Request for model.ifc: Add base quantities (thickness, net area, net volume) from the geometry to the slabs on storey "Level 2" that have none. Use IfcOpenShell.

First a look at what the model holds.

```python
import ifcopenshell
import ifcopenshell.util.element
import ifcopenshell.util.unit

model = ifcopenshell.open("model.ifc")
print(model.schema)
for unit_type in ("LENGTHUNIT", "AREAUNIT", "VOLUMEUNIT"):
    print(unit_type, ifcopenshell.util.unit.calculate_unit_scale(model, unit_type))
storey = next(s for s in model.by_type("IfcBuildingStorey") if s.Name == "Level 2")
slabs = [e for e in ifcopenshell.util.element.get_decomposition(storey) if e.is_a("IfcSlab")]
for e in sorted(slabs, key=lambda e: e.id()):
    print(e.id(), e.is_a(), e.Name, list(ifcopenshell.util.element.get_psets(e, qtos_only=True)), sep=" | ")
```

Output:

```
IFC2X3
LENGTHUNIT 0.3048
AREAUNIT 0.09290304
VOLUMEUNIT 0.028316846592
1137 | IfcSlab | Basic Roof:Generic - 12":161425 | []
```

```python
import ifcopenshell
import ifcopenshell.api.pset
import ifcopenshell.geom
import ifcopenshell.util.element
import ifcopenshell.util.shape
import ifcopenshell.util.unit

model = ifcopenshell.open("model.ifc")
unit_scale = ifcopenshell.util.unit.calculate_unit_scale(model)
area_scale = ifcopenshell.util.unit.calculate_unit_scale(model, "AREAUNIT")
volume_scale = ifcopenshell.util.unit.calculate_unit_scale(model, "VOLUMEUNIT")
settings = ifcopenshell.geom.settings()

storey = next(s for s in model.by_type("IfcBuildingStorey") if s.Name == "Level 2")
slabs = [e for e in ifcopenshell.util.element.get_decomposition(storey) if e.is_a("IfcSlab")]

for e in sorted(slabs, key=lambda e: e.id()):
    if ifcopenshell.util.element.get_psets(e, qtos_only=True, should_inherit=False):
        continue
    # Geometry comes back in metres, in the element's own axes.
    shape = ifcopenshell.geom.create_shape(settings, e)
    values = {
        "Width": ifcopenshell.util.shape.get_z(shape.geometry) / unit_scale,
        "NetArea": ifcopenshell.util.shape.get_footprint_area(shape.geometry) / area_scale,
        "NetVolume": ifcopenshell.util.shape.get_volume(shape.geometry) / volume_scale,
    }
    qto = ifcopenshell.api.pset.add_qto(model, product=e, name="BaseQuantities")
    ifcopenshell.api.pset.edit_qto(model, qto=qto, properties=values)
    print(e.id(), {k: round(v, 3) for k, v in values.items()})

model.write("model-out.ifc")
```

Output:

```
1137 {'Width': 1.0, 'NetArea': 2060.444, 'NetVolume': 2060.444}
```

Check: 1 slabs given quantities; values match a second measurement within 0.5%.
